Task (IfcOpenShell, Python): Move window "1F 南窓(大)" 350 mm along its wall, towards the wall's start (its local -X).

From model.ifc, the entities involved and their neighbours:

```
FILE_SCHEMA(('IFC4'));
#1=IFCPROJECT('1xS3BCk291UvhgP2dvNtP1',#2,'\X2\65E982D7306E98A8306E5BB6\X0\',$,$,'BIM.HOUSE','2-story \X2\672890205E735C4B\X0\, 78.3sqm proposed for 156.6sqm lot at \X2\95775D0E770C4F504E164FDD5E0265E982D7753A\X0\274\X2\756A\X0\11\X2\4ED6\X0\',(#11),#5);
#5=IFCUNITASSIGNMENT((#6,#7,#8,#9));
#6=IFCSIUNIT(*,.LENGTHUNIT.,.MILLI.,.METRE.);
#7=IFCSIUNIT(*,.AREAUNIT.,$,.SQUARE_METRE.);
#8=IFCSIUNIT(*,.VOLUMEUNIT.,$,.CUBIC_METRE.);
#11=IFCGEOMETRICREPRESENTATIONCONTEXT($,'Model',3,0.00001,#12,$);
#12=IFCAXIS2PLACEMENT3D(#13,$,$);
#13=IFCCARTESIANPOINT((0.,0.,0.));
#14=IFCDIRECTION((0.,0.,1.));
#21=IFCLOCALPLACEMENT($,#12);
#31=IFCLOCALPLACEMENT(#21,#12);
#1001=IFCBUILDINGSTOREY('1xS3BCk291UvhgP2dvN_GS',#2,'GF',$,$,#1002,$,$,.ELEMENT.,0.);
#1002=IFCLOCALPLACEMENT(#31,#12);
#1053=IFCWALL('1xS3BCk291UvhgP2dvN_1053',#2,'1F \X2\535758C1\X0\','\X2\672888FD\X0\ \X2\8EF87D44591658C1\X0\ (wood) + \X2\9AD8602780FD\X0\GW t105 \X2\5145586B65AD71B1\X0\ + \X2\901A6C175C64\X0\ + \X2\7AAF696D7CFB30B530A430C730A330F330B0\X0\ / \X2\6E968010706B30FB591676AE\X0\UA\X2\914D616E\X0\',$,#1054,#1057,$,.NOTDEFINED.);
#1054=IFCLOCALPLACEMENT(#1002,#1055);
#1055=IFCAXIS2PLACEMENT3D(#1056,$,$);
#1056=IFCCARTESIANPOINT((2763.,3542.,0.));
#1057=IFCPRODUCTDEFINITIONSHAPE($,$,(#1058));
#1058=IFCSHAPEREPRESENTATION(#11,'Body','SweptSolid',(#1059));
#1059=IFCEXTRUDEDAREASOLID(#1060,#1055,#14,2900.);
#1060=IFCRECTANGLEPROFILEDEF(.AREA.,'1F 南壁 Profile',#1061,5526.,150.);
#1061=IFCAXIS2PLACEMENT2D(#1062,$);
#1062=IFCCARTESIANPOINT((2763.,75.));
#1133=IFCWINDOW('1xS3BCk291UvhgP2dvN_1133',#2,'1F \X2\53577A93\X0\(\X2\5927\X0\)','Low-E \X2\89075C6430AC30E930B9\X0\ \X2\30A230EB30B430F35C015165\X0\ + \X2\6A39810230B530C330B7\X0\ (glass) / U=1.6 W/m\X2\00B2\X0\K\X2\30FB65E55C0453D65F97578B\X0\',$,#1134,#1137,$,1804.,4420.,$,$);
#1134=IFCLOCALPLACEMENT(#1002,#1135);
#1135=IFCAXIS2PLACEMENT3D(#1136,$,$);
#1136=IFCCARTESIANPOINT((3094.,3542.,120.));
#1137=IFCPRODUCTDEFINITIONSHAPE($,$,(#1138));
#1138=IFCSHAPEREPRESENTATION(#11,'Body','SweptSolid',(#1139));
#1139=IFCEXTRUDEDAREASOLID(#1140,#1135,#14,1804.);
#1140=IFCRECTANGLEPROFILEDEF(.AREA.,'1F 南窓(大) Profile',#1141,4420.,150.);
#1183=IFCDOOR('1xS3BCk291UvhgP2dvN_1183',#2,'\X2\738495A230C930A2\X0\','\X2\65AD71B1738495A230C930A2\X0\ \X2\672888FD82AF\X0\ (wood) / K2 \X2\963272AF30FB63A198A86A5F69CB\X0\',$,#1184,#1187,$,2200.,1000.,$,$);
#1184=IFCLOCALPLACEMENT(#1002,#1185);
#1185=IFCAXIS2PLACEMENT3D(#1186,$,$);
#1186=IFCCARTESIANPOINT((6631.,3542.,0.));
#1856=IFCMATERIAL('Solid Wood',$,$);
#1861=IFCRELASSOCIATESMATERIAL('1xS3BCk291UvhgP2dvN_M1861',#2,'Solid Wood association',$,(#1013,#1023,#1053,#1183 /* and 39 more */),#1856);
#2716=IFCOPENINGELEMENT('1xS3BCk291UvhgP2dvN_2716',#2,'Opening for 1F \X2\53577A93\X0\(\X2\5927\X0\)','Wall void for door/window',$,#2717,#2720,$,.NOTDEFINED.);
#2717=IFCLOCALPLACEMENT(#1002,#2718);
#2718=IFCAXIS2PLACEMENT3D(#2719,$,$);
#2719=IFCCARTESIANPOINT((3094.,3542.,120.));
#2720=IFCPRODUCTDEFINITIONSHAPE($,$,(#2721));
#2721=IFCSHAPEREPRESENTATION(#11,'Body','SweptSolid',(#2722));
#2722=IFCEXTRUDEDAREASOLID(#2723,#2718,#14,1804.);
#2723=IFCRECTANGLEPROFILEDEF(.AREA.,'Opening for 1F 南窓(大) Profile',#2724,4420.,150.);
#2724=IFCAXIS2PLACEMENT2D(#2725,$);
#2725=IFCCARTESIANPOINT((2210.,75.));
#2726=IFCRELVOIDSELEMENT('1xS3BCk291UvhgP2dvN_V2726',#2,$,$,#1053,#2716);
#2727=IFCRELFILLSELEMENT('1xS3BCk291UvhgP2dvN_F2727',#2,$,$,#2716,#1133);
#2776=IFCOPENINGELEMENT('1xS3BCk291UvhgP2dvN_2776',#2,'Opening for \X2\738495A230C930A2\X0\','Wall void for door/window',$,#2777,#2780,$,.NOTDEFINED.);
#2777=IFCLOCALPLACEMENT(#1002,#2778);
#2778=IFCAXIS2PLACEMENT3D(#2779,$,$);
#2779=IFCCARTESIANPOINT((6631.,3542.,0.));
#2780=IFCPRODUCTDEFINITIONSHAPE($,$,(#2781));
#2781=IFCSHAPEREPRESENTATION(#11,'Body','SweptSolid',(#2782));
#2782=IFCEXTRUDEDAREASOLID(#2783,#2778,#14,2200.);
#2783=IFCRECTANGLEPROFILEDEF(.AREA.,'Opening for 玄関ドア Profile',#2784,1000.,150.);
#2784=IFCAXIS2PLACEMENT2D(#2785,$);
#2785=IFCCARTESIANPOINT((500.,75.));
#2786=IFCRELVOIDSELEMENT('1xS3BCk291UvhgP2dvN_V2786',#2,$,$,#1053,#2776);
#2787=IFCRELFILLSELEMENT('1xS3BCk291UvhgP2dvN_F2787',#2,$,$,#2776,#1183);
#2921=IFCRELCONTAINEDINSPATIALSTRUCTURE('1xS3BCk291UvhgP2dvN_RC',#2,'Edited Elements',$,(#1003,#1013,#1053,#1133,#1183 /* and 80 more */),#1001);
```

```python
import ifcopenshell
import ifcopenshell.api.geometry
import ifcopenshell.util.placement

model = ifcopenshell.open("model.ifc")

window = model.by_guid("1xS3BCk291UvhgP2dvN_1133")
opening = window.FillsVoids[0].RelatingOpeningElement
wall = opening.VoidsElements[0].RelatingBuildingElement

wall_matrix = ifcopenshell.util.placement.get_local_placement(wall.ObjectPlacement)
shift = wall_matrix[:3, 0] * -350.0
before = ifcopenshell.util.placement.get_local_placement(window.ObjectPlacement)[:3, 3].copy()

# The window is not placed relative to its opening, so move both.
for product in (opening, window):
    matrix = ifcopenshell.util.placement.get_local_placement(product.ObjectPlacement)
    matrix[:3, 3] += shift
    ifcopenshell.api.geometry.edit_object_placement(model, product=product, matrix=matrix, is_si=False)

after = ifcopenshell.util.placement.get_local_placement(window.ObjectPlacement)[:3, 3]
print("window moved by", (after - before).round(3) + 0.0)

model.write("model_edited.ifc")
```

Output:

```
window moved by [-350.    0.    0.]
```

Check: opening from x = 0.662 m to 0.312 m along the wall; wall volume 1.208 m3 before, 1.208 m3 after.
